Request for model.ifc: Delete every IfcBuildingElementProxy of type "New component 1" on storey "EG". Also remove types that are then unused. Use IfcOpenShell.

First a look at what the model holds.

```python
import ifcopenshell
import ifcopenshell.util.element

model = ifcopenshell.open("model.ifc")
print(model.schema)
storey = next(s for s in model.by_type("IfcBuildingStorey") if s.Name == "EG")
proxies = [e for e in ifcopenshell.util.element.get_decomposition(storey) if e.is_a("IfcBuildingElementProxy")]
seen = {}
for e in proxies:
    element_type = ifcopenshell.util.element.get_type(e)
    name = element_type.Name if element_type not in (None, e) else None
    seen[name] = seen.get(name, 0) + 1
for name, count in sorted(seen.items(), key=str):
    print(count, "x", name)
```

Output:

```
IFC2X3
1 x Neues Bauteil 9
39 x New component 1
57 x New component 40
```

```python
import ifcopenshell
import ifcopenshell.api.root
import ifcopenshell.util.element

model = ifcopenshell.open("model.ifc")

storey = next(s for s in model.by_type("IfcBuildingStorey") if s.Name == "EG")
proxies = [e for e in ifcopenshell.util.element.get_decomposition(storey) if e.is_a("IfcBuildingElementProxy")]
targets = [e for e in proxies if (t := ifcopenshell.util.element.get_type(e)) not in (None, e) and t.Name == "New component 1"]
types = {ifcopenshell.util.element.get_type(e) for e in targets} - {None, *targets}

for e in targets:
    ifcopenshell.api.root.remove_product(model, product=e)
print(len(targets), "removed")

unused = [t for t in types if not ifcopenshell.util.element.get_types(t)]
for t in unused:
    ifcopenshell.api.root.remove_product(model, product=t)
print(len(unused), "unused types removed")

model.write("model_v2.ifc")
```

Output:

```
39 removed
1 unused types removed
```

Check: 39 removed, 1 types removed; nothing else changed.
